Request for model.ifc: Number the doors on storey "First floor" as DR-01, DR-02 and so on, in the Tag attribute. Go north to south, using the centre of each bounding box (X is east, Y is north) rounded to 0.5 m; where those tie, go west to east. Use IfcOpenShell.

First a look at what the model holds.

```python
import ifcopenshell
import ifcopenshell.util.element
import ifcopenshell.util.placement

model = ifcopenshell.open("model.ifc")
print(model.schema)
storey = next(s for s in model.by_type("IfcBuildingStorey") if s.Name == "First floor")
doors = [e for e in ifcopenshell.util.element.get_decomposition(storey) if e.is_a("IfcDoor")]
for e in sorted(doors, key=lambda e: e.id()):
    origin = ifcopenshell.util.placement.get_local_placement(e.ObjectPlacement)[:3, 3]
    print(e.id(), e.Tag, e.Name, origin.round(2) + 0.0, sep=" | ")
```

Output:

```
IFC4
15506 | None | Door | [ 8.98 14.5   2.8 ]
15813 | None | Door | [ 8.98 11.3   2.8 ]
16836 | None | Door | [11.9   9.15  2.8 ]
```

```python
import ifcopenshell
import ifcopenshell.geom
import ifcopenshell.util.element
import ifcopenshell.util.shape

model = ifcopenshell.open("model.ifc")
settings = ifcopenshell.geom.settings()
settings.set("use-world-coords", True)


def centre(element):
    shape = ifcopenshell.geom.create_shape(settings, element)
    return ifcopenshell.util.shape.get_bbox_centroid(shape.geometry)


storey = next(s for s in model.by_type("IfcBuildingStorey") if s.Name == "First floor")
doors = [e for e in ifcopenshell.util.element.get_decomposition(storey) if e.is_a("IfcDoor")]

# Insertion points can sit at a corner or the storey origin, so sort by the geometry (in metres).
centres = {e: centre(e) for e in doors}
doors.sort(key=lambda e: (-round(centres[e][1] / 0.5), centres[e][0]))

for i, e in enumerate(doors, start=1):
    number = f"DR-{i:02d}"
    e.Tag = number
    print(e.id(), number)

model.write("model_v2.ifc")
```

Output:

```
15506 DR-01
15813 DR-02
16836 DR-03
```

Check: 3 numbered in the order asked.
